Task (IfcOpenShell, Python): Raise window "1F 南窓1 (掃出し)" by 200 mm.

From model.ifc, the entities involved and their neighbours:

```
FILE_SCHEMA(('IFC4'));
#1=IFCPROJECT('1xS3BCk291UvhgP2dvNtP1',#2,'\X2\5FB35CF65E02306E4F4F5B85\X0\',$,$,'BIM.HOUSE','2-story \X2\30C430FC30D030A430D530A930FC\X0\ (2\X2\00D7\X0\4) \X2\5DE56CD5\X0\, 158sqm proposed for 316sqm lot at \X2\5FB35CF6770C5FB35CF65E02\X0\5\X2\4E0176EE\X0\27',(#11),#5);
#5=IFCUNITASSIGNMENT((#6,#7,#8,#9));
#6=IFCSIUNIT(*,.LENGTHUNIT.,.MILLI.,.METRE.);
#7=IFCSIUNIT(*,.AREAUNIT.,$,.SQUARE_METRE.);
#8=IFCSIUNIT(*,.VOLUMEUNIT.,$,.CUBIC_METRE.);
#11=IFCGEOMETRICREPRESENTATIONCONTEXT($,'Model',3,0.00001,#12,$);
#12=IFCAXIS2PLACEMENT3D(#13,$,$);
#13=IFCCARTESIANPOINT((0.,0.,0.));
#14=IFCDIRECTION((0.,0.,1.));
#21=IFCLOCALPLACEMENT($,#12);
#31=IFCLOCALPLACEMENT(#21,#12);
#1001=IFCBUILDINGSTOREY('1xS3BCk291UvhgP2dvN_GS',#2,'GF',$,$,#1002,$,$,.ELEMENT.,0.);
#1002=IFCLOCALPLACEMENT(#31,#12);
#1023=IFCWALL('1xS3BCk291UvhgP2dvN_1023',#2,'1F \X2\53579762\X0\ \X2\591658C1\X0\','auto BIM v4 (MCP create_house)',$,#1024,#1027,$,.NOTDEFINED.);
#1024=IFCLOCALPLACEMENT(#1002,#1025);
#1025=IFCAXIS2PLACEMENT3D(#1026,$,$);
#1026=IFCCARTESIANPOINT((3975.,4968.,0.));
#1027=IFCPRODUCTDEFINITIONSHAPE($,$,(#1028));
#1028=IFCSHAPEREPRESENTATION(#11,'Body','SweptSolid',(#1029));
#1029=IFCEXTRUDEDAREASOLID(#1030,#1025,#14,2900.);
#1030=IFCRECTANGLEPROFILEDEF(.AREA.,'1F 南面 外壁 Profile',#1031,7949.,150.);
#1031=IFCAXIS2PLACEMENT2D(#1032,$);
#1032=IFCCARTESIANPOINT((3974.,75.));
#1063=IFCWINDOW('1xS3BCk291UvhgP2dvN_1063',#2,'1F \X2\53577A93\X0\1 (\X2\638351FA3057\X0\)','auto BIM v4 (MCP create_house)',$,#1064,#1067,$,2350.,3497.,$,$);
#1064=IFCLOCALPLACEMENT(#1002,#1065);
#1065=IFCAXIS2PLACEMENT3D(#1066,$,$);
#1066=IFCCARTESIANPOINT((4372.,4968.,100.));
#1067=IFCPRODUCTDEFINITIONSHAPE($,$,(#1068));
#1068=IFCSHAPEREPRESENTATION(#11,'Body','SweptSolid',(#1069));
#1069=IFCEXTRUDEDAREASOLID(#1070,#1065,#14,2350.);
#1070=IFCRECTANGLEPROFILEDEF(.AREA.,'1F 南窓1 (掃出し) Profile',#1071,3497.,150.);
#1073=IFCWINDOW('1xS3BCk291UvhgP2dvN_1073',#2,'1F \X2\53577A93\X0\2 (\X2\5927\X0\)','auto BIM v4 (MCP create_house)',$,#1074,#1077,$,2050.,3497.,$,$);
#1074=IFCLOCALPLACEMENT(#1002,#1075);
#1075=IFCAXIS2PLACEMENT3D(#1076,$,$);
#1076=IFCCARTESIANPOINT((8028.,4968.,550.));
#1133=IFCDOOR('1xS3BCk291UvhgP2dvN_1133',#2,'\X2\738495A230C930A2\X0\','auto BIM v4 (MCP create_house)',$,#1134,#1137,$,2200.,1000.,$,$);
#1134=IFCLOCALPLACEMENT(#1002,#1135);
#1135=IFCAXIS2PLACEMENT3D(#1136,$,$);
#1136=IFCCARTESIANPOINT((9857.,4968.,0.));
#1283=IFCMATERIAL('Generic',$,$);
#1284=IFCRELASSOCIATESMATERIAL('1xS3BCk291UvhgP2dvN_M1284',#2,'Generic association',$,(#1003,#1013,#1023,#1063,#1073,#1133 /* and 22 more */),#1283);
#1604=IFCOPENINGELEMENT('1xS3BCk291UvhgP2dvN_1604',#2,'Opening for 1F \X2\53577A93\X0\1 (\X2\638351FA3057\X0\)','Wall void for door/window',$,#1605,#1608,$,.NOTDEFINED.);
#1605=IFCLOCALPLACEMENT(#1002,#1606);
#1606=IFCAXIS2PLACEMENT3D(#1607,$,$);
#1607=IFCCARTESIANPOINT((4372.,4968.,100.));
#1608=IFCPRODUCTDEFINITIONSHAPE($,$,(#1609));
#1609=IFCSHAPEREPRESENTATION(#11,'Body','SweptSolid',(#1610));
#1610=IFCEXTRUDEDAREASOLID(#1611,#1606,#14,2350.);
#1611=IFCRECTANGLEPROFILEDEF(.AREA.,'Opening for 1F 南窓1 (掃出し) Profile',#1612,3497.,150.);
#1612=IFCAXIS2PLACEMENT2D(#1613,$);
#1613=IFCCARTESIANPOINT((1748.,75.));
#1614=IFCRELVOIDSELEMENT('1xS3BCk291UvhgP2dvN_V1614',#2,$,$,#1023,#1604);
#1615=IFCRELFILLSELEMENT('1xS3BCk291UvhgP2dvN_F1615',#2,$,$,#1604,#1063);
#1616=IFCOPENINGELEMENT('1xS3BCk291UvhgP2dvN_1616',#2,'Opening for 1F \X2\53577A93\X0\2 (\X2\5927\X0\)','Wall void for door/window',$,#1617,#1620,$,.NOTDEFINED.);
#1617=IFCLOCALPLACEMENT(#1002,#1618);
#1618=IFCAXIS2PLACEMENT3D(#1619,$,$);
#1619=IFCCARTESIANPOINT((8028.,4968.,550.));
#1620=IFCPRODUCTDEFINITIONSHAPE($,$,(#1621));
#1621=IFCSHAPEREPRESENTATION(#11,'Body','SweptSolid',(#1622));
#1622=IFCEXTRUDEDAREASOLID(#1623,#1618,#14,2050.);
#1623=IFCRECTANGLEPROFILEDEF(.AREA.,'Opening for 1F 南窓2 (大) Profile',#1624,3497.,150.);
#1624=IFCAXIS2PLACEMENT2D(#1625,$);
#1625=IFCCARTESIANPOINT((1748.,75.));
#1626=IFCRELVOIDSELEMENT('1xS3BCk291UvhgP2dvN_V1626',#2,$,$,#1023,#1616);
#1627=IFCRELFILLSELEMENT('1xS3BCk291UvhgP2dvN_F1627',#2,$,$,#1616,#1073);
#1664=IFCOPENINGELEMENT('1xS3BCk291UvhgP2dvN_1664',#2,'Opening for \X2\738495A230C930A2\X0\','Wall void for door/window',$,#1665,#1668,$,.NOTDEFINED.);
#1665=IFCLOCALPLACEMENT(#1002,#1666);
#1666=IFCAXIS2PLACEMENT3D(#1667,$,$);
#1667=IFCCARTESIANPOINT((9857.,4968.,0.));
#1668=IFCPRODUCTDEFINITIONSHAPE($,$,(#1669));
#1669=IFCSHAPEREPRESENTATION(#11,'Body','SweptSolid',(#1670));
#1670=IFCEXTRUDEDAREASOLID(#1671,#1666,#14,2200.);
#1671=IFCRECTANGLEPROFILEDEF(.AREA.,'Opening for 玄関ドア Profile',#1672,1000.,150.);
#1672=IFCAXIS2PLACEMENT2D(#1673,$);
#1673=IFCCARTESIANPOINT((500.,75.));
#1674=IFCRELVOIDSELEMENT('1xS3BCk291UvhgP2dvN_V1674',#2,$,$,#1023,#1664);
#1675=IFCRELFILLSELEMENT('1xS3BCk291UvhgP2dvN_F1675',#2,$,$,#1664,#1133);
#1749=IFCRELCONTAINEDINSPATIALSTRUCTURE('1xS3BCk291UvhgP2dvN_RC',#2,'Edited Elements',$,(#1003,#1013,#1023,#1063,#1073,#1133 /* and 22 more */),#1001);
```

```python
import numpy as np
import ifcopenshell
import ifcopenshell.api.geometry
import ifcopenshell.util.placement
import ifcopenshell.util.unit

model = ifcopenshell.open("model.ifc")
unit_scale = ifcopenshell.util.unit.calculate_unit_scale(model)

window = model.by_guid("1xS3BCk291UvhgP2dvN_1063")
opening = window.FillsVoids[0].RelatingOpeningElement
dz = 0.2 / unit_scale

shift = np.array([0.0, 0.0, dz])
# The window is not placed relative to its opening, so move both.
for product in (opening, window):
    matrix = ifcopenshell.util.placement.get_local_placement(product.ObjectPlacement)
    matrix[:3, 3] += shift
    ifcopenshell.api.geometry.edit_object_placement(model, product=product, matrix=matrix, is_si=False)

print(f"moved by {dz * unit_scale:+.3f} m")

model.write("model_edited.ifc")
```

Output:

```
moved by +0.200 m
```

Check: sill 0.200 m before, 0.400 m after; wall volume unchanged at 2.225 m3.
